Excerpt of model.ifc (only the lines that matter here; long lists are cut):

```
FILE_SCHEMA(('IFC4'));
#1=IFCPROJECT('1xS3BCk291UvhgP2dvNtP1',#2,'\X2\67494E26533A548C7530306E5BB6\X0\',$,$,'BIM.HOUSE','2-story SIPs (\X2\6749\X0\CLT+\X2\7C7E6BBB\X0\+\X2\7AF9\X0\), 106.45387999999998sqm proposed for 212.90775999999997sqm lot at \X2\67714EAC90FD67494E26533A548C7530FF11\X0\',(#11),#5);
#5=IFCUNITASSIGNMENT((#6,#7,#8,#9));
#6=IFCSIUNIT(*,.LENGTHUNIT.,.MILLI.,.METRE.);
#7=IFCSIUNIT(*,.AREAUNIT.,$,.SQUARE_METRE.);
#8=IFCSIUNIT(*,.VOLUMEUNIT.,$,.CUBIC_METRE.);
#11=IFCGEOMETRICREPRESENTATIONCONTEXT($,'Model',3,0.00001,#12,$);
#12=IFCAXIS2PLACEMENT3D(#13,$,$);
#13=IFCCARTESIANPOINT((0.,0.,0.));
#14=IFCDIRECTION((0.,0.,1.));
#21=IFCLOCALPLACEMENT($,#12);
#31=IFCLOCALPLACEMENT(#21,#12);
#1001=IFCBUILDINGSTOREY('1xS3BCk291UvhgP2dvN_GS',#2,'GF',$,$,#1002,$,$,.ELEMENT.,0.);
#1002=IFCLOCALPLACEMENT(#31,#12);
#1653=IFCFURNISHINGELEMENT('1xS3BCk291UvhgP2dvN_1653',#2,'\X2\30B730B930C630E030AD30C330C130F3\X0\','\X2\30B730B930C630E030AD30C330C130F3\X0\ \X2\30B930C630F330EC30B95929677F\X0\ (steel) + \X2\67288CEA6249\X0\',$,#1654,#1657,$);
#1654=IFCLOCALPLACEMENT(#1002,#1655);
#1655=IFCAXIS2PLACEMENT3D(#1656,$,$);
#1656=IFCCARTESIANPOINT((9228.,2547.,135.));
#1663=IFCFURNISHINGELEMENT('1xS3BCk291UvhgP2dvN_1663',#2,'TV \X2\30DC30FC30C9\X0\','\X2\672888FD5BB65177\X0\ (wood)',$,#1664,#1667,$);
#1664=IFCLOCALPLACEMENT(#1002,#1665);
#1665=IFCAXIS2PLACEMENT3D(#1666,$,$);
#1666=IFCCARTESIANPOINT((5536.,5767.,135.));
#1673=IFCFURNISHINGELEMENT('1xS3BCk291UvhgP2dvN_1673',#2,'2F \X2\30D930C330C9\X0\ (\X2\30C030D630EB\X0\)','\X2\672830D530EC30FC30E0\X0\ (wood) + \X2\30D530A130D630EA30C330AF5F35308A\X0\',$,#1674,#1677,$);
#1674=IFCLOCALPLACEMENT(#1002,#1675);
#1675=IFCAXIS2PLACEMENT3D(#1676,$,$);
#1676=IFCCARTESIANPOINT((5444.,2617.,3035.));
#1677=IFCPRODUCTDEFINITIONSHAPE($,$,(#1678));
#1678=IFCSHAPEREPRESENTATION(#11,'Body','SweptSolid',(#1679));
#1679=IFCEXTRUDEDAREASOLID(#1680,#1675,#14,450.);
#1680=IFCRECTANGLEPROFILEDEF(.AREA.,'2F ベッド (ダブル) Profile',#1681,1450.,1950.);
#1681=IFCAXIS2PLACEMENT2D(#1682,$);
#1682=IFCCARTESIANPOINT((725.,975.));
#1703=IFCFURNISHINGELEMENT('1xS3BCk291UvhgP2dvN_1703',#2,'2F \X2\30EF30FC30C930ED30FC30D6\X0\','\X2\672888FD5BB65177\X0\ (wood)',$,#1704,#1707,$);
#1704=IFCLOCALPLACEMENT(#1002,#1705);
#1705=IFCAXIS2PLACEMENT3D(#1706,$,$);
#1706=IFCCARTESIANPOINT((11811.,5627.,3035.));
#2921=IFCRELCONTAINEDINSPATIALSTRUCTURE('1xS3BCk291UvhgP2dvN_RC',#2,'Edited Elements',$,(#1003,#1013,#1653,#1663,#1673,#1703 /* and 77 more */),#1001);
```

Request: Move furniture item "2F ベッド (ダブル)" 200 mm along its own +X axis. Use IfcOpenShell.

```python
import ifcopenshell
import ifcopenshell.api.geometry
import ifcopenshell.util.placement
import ifcopenshell.util.unit

model = ifcopenshell.open("model.ifc")
unit_scale = ifcopenshell.util.unit.calculate_unit_scale(model)

item = model.by_guid("1xS3BCk291UvhgP2dvN_1673")
matrix = ifcopenshell.util.placement.get_local_placement(item.ObjectPlacement)
matrix[:3, 3] += matrix[:3, 0] * 0.2 / unit_scale
ifcopenshell.api.geometry.edit_object_placement(model, product=item, matrix=matrix, is_si=False)

print(ifcopenshell.util.placement.get_local_placement(item.ObjectPlacement).round(3) + 0.0)

model.write("model_rev.ifc")
```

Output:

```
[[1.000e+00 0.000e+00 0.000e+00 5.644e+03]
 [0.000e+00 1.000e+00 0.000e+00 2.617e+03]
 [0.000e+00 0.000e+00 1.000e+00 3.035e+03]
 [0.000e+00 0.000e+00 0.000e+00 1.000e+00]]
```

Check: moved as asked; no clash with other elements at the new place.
